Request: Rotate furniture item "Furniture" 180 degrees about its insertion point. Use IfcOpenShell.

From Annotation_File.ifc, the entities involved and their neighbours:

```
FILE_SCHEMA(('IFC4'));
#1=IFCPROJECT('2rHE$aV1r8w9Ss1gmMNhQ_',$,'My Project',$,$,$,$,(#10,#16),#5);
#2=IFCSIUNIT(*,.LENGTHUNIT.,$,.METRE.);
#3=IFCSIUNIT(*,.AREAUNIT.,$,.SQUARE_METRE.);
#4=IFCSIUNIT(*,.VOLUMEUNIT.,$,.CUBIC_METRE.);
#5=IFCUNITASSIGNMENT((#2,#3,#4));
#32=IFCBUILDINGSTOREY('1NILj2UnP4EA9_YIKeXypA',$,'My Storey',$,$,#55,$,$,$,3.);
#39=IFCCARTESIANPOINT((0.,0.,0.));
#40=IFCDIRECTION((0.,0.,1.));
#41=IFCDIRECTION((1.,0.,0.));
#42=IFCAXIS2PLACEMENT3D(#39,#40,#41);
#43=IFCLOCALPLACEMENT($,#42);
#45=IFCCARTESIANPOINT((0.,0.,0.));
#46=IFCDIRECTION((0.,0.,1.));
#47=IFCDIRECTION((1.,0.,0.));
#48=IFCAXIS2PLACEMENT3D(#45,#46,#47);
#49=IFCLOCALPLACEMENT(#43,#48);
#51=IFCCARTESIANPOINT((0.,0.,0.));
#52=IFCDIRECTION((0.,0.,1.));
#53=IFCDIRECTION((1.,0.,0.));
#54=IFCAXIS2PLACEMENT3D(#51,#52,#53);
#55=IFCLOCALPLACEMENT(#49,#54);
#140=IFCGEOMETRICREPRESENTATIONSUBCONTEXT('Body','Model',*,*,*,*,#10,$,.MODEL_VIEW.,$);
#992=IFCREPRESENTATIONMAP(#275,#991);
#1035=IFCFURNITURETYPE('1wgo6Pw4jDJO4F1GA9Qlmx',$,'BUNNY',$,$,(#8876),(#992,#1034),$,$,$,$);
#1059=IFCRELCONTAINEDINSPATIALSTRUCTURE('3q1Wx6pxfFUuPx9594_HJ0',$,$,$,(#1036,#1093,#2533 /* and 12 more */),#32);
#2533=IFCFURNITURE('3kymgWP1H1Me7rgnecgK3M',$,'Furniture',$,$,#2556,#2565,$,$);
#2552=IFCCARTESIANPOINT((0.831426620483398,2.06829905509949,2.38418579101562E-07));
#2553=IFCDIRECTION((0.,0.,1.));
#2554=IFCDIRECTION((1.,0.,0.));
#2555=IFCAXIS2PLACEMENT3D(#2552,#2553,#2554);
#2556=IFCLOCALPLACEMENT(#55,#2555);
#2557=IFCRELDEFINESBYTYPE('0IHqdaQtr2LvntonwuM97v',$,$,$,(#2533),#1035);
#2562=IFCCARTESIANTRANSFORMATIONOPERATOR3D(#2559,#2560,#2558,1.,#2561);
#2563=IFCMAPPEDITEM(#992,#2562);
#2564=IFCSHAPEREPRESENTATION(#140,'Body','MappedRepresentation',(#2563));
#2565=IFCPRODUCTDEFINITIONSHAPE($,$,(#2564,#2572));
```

```python
import ifcopenshell
import ifcopenshell.api.geometry
import ifcopenshell.util.placement

model = ifcopenshell.open("Annotation_File.ifc")

item = model.by_guid("3kymgWP1H1Me7rgnecgK3M")
matrix = ifcopenshell.util.placement.get_local_placement(item.ObjectPlacement)
matrix = matrix @ ifcopenshell.util.placement.rotation(180, "Z")
ifcopenshell.api.geometry.edit_object_placement(model, product=item, matrix=matrix, is_si=False)

print(ifcopenshell.util.placement.get_local_placement(item.ObjectPlacement).round(3) + 0.0)

model.write("Annotation_File_rev.ifc")
```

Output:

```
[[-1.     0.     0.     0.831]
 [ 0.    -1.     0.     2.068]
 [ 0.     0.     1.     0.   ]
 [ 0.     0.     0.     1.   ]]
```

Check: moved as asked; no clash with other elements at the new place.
